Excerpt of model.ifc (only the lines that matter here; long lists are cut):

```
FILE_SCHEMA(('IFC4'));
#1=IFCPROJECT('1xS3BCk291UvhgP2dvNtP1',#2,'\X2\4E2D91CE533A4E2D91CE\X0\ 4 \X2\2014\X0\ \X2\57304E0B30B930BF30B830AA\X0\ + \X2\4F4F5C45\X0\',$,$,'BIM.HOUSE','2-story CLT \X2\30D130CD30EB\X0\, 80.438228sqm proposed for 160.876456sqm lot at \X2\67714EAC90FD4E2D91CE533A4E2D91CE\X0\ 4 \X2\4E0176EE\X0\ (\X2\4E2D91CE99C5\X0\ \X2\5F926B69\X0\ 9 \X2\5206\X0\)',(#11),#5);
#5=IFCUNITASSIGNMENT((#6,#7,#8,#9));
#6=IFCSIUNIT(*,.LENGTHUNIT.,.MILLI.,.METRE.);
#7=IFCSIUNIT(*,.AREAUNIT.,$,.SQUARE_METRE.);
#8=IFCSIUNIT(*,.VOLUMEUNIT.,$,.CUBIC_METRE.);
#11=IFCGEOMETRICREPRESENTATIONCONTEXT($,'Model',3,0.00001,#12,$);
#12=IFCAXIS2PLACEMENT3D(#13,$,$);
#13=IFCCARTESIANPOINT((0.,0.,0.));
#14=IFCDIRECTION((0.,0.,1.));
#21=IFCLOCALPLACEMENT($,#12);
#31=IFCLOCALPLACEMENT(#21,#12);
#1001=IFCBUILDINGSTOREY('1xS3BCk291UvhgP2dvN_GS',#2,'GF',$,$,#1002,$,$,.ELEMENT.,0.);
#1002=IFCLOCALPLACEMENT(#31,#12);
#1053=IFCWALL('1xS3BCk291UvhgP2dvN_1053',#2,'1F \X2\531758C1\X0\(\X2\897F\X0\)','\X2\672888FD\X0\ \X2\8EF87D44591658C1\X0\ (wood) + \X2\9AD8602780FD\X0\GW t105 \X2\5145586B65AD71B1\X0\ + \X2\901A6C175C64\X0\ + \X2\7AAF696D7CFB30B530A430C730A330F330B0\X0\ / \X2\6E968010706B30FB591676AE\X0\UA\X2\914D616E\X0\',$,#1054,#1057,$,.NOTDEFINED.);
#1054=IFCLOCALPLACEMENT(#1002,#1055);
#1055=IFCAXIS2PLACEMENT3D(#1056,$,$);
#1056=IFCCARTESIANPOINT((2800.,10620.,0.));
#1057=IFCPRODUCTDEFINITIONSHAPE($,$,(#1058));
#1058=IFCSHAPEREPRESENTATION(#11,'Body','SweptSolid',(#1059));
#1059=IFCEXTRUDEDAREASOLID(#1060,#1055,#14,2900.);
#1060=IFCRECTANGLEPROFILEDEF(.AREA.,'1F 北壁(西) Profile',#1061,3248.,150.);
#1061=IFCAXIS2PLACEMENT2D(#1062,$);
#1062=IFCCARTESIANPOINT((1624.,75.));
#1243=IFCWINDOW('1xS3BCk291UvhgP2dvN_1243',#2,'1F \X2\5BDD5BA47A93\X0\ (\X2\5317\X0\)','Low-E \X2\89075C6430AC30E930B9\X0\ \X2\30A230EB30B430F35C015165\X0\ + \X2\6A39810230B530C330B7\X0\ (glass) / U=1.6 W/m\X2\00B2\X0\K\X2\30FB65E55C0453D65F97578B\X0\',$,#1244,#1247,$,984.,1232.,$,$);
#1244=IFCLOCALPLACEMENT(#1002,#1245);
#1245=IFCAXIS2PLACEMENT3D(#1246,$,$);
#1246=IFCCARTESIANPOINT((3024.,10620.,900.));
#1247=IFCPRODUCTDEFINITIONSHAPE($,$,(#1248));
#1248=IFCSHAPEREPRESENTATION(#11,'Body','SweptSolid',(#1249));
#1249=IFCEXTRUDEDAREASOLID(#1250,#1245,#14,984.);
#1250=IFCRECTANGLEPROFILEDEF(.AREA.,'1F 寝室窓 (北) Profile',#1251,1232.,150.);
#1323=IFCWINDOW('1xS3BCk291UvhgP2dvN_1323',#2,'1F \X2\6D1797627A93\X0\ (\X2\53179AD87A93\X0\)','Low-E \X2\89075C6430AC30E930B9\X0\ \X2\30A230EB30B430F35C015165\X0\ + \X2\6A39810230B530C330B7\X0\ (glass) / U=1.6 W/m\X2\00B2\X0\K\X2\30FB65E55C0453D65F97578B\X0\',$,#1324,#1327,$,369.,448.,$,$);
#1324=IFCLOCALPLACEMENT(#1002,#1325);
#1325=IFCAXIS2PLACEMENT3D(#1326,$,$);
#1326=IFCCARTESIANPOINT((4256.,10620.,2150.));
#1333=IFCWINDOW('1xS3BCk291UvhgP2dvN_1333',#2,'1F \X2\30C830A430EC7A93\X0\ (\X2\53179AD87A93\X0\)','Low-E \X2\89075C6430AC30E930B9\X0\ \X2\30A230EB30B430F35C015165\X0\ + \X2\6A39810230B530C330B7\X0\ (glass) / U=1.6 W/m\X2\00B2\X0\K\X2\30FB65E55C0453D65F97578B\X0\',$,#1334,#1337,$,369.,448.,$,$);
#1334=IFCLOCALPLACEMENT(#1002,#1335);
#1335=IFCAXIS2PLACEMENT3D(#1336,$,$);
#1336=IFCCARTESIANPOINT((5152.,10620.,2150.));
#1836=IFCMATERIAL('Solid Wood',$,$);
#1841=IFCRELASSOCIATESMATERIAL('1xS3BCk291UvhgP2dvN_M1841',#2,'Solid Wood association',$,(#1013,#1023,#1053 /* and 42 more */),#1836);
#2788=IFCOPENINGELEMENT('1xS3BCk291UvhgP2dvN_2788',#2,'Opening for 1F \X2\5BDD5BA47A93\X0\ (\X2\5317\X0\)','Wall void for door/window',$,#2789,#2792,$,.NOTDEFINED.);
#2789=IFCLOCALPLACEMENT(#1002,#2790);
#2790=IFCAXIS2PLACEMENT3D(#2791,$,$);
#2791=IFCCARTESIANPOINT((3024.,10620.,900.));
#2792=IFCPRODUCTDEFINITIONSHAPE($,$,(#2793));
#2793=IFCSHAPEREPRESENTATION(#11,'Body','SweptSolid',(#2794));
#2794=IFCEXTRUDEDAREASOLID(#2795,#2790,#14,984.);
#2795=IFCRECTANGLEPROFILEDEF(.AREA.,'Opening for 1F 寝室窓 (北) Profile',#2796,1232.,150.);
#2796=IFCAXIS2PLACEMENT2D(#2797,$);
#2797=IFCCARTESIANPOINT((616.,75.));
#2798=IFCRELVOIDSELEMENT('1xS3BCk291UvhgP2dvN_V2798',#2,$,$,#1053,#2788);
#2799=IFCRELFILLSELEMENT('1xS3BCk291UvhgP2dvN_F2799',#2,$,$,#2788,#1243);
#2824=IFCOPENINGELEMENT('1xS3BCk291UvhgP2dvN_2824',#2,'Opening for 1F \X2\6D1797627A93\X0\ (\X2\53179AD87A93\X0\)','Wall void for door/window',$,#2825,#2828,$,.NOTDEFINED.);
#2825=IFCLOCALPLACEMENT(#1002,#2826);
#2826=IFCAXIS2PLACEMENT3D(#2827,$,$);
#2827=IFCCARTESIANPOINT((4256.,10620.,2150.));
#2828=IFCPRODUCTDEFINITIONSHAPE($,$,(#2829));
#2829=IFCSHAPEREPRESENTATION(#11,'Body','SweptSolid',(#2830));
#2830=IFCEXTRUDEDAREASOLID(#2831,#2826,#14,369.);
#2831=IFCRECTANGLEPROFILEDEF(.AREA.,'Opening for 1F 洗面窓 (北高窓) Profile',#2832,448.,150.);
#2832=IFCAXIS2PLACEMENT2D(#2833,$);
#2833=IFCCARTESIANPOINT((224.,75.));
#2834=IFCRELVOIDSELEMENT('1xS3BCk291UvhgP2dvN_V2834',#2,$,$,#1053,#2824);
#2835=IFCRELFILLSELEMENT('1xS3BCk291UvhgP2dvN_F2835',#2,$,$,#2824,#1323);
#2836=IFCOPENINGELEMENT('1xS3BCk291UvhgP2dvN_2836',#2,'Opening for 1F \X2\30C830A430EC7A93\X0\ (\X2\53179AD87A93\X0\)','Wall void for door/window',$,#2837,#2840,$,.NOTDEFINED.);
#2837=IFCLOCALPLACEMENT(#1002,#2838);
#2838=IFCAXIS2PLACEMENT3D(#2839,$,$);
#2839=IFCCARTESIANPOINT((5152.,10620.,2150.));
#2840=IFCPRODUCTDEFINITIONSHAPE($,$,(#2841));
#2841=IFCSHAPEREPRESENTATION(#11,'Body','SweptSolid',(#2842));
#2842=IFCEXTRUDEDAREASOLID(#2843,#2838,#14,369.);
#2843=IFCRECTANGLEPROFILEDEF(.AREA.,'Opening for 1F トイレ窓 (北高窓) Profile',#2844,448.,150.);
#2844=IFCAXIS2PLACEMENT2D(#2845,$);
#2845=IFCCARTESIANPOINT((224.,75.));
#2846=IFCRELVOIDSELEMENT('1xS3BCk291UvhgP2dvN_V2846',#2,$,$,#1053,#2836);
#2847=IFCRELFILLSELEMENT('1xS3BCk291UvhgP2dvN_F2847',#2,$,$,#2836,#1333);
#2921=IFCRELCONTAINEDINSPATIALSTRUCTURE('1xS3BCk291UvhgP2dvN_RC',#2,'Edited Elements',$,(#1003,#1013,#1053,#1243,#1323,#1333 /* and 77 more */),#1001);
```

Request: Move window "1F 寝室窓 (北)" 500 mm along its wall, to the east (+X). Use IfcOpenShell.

```python
import ifcopenshell
import ifcopenshell.api.geometry
import ifcopenshell.util.placement

model = ifcopenshell.open("model.ifc")

window = model.by_guid("1xS3BCk291UvhgP2dvN_1243")
opening = window.FillsVoids[0].RelatingOpeningElement
wall = opening.VoidsElements[0].RelatingBuildingElement

wall_matrix = ifcopenshell.util.placement.get_local_placement(wall.ObjectPlacement)
shift = wall_matrix[:3, 0] * 500.0
before = ifcopenshell.util.placement.get_local_placement(window.ObjectPlacement)[:3, 3].copy()

# The window is not placed relative to its opening, so move both.
for product in (opening, window):
    matrix = ifcopenshell.util.placement.get_local_placement(product.ObjectPlacement)
    matrix[:3, 3] += shift
    ifcopenshell.api.geometry.edit_object_placement(model, product=product, matrix=matrix, is_si=False)

after = ifcopenshell.util.placement.get_local_placement(window.ObjectPlacement)[:3, 3]
print("window moved by", (after - before).round(3) + 0.0)

model.write("model_updated.ifc")
```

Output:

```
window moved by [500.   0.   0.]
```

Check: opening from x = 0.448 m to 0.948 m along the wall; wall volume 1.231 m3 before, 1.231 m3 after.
